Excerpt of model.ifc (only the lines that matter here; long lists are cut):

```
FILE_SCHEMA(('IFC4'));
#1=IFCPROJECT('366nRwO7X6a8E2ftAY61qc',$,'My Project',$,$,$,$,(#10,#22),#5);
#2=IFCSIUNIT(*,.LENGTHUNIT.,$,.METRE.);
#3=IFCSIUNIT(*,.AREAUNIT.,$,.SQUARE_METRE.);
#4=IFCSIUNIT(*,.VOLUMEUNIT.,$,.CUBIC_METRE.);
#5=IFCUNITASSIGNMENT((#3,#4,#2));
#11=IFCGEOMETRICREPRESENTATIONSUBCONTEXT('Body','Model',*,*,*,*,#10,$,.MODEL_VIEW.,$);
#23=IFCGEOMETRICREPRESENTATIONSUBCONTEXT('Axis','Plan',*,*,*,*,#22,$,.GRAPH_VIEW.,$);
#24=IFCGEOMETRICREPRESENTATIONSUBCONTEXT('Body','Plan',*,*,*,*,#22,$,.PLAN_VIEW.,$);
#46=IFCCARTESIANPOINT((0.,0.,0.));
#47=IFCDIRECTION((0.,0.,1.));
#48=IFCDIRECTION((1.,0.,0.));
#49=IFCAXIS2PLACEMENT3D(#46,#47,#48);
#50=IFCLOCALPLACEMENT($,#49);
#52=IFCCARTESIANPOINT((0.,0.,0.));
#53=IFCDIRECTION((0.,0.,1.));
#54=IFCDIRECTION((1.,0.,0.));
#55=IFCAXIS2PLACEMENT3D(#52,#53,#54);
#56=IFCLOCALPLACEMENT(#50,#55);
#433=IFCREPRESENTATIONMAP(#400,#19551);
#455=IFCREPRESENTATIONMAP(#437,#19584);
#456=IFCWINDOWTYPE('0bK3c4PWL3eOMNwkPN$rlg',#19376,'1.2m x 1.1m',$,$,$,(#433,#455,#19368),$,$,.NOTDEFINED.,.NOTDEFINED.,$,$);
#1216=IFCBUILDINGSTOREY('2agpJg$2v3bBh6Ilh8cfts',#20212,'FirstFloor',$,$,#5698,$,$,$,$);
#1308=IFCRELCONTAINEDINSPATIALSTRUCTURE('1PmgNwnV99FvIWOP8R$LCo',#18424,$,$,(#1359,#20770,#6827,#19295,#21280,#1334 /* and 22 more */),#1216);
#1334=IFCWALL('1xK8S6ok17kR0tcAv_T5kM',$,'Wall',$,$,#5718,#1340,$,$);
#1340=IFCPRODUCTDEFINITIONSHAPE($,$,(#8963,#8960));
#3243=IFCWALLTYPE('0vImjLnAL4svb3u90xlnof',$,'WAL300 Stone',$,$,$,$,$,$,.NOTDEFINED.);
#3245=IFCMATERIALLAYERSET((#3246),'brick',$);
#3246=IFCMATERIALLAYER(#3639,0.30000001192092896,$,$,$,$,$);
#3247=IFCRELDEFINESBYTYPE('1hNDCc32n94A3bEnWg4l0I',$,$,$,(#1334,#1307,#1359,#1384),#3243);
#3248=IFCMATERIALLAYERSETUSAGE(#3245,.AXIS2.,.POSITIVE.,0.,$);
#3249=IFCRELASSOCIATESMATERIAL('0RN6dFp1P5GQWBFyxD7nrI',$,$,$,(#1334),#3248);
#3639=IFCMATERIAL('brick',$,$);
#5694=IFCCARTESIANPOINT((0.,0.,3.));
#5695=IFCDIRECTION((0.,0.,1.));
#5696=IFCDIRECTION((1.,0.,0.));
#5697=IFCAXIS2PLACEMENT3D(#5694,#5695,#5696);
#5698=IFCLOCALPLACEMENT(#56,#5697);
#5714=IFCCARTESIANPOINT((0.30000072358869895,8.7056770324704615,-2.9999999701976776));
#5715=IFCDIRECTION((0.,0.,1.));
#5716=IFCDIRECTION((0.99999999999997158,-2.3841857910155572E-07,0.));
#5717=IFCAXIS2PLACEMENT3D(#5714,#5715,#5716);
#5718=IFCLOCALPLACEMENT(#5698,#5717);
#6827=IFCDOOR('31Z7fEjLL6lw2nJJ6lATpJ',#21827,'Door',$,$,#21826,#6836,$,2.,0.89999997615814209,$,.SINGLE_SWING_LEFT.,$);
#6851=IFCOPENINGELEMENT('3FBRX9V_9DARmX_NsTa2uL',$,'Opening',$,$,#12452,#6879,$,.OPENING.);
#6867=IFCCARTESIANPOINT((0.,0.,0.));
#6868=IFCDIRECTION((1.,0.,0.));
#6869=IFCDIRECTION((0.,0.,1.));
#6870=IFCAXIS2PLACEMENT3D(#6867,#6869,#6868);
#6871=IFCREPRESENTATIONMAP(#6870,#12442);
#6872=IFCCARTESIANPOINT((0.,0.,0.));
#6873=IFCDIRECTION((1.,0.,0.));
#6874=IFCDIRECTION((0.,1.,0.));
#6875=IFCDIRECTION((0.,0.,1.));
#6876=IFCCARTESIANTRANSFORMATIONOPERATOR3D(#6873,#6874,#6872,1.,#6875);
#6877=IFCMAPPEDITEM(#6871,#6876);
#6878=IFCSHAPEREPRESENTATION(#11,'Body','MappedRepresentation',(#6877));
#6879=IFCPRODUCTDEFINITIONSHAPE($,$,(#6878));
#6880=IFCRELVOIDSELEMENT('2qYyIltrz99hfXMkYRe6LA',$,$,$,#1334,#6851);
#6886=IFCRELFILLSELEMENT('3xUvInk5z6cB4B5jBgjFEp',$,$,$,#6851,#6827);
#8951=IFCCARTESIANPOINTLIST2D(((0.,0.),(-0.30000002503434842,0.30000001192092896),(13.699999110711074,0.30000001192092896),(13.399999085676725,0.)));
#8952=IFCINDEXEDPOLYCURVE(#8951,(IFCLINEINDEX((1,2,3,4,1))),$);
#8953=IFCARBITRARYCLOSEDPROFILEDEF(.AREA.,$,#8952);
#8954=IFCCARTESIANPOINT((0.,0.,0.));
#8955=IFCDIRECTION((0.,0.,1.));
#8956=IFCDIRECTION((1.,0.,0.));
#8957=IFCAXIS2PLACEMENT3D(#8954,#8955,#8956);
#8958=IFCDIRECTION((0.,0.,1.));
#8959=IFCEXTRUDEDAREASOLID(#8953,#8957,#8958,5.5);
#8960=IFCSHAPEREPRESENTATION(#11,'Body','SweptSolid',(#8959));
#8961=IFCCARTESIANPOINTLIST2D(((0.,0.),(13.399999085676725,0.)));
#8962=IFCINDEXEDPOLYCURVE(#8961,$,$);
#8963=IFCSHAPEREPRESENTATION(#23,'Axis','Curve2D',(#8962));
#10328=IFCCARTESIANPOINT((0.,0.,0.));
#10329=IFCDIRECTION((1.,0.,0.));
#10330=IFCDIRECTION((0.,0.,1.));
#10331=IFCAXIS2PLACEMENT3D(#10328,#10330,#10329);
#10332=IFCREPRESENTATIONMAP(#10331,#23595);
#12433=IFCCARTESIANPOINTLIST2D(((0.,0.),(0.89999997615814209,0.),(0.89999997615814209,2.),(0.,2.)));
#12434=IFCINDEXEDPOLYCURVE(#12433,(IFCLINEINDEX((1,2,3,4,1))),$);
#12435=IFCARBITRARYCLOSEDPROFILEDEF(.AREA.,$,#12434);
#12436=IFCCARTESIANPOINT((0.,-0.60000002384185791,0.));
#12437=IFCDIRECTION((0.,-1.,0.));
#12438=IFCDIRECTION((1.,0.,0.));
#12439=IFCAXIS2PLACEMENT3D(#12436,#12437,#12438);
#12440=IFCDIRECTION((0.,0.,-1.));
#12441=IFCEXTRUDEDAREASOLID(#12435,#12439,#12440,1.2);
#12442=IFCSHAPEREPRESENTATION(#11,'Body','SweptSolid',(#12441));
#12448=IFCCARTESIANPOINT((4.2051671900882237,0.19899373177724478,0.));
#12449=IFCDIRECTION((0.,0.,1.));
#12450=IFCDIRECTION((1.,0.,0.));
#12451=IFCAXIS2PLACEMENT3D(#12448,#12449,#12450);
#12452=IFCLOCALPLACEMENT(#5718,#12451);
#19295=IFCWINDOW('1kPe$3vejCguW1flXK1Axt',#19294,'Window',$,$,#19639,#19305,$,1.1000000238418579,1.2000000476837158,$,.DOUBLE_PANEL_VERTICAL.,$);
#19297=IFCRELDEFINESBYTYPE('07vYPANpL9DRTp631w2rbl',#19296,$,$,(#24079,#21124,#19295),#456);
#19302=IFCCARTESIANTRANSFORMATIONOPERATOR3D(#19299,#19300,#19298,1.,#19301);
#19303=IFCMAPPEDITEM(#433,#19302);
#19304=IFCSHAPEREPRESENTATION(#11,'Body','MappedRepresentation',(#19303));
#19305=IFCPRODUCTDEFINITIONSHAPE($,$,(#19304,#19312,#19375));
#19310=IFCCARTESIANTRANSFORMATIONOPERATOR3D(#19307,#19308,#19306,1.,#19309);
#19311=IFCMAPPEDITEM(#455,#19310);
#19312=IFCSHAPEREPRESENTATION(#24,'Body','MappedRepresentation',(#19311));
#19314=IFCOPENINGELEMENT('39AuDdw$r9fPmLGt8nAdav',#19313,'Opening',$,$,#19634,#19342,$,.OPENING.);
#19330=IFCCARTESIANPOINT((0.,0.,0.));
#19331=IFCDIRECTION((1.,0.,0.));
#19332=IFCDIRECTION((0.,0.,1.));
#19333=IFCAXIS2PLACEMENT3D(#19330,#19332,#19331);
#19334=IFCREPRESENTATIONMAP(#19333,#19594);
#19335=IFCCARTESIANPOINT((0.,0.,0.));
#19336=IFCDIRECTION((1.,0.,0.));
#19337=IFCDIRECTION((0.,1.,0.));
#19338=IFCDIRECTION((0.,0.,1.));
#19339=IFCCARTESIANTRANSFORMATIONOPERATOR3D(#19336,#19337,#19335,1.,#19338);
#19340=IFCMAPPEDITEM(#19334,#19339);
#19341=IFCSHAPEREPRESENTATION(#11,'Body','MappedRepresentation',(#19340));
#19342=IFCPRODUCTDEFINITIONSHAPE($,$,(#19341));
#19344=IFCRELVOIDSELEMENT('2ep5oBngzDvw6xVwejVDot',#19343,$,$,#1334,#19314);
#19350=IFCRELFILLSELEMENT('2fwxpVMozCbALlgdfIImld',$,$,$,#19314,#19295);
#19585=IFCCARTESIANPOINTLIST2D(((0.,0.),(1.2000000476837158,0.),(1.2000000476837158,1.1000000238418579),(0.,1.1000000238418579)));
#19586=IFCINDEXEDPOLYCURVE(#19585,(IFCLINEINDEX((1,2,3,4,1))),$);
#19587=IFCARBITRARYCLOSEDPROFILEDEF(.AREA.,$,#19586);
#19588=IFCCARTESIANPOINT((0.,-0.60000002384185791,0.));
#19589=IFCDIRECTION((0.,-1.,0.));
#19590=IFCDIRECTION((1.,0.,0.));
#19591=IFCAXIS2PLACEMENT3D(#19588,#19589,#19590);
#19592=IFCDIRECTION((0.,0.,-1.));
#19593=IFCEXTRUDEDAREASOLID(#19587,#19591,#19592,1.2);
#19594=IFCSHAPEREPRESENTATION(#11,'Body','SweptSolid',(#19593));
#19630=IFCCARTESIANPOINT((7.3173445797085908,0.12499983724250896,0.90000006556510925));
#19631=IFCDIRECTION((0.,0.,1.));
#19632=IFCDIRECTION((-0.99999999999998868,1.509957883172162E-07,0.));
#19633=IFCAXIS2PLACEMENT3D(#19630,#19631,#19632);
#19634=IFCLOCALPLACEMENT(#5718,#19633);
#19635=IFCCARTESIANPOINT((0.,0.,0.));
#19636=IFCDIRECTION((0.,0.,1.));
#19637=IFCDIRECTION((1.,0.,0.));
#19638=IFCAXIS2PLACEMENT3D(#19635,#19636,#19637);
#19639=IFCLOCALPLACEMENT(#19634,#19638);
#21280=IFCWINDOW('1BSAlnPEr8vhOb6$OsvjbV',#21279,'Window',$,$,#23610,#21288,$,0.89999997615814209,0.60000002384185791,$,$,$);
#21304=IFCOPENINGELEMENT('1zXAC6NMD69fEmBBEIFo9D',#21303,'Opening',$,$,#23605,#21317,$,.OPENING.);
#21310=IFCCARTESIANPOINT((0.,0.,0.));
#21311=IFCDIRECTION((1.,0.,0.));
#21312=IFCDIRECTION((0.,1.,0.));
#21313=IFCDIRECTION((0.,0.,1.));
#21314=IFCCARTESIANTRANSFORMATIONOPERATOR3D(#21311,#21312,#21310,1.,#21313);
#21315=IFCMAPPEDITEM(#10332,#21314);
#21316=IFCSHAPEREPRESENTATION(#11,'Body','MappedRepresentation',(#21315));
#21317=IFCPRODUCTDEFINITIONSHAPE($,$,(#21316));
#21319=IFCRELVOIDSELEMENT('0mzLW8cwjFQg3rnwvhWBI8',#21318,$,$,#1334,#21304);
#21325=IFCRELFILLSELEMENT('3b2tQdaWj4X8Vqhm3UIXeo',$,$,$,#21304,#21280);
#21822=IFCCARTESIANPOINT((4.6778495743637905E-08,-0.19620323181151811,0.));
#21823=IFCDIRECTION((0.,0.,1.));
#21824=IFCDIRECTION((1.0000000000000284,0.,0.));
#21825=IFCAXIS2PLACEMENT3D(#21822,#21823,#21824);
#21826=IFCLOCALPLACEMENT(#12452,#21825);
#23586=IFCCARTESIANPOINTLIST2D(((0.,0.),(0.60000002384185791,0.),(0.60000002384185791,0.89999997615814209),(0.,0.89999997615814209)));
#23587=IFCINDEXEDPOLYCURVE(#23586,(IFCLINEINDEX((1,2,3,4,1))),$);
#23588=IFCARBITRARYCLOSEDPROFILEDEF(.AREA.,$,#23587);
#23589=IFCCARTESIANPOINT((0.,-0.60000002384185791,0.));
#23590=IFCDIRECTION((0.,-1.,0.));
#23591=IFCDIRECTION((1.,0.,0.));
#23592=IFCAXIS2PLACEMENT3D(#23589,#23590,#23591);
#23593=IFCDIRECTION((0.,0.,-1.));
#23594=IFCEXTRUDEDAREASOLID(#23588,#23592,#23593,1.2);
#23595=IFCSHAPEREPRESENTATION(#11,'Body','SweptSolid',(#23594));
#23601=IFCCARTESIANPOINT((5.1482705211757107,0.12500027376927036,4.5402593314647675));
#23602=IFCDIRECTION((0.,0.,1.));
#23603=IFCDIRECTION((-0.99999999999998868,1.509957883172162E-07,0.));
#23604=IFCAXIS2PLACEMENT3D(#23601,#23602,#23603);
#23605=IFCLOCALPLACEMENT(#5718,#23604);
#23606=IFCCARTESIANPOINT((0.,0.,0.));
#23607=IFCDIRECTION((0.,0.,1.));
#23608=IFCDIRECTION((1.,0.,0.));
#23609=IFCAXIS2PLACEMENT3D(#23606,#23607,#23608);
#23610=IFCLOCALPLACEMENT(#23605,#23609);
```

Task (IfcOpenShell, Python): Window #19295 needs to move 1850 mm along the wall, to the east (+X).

```python
import ifcopenshell
import ifcopenshell.api.geometry
import ifcopenshell.util.placement

model = ifcopenshell.open("model.ifc")

window = model.by_guid("1kPe$3vejCguW1flXK1Axt")
opening = window.FillsVoids[0].RelatingOpeningElement
wall = opening.VoidsElements[0].RelatingBuildingElement

wall_matrix = ifcopenshell.util.placement.get_local_placement(wall.ObjectPlacement)
shift = wall_matrix[:3, 0] * 1.85
before = ifcopenshell.util.placement.get_local_placement(window.ObjectPlacement)[:3, 3].copy()

# The window is placed relative to its opening, so it follows when the opening moves.
matrix = ifcopenshell.util.placement.get_local_placement(opening.ObjectPlacement)
matrix[:3, 3] += shift
ifcopenshell.api.geometry.edit_object_placement(
    model, product=opening, matrix=matrix, is_si=False, should_transform_children=True
)

after = ifcopenshell.util.placement.get_local_placement(window.ObjectPlacement)[:3, 3]
print("window moved by", (after - before).round(3) + 0.0)

model.write("model_rev.ifc")
```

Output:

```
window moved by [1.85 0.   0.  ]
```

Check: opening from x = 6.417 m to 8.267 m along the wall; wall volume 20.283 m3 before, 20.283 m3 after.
